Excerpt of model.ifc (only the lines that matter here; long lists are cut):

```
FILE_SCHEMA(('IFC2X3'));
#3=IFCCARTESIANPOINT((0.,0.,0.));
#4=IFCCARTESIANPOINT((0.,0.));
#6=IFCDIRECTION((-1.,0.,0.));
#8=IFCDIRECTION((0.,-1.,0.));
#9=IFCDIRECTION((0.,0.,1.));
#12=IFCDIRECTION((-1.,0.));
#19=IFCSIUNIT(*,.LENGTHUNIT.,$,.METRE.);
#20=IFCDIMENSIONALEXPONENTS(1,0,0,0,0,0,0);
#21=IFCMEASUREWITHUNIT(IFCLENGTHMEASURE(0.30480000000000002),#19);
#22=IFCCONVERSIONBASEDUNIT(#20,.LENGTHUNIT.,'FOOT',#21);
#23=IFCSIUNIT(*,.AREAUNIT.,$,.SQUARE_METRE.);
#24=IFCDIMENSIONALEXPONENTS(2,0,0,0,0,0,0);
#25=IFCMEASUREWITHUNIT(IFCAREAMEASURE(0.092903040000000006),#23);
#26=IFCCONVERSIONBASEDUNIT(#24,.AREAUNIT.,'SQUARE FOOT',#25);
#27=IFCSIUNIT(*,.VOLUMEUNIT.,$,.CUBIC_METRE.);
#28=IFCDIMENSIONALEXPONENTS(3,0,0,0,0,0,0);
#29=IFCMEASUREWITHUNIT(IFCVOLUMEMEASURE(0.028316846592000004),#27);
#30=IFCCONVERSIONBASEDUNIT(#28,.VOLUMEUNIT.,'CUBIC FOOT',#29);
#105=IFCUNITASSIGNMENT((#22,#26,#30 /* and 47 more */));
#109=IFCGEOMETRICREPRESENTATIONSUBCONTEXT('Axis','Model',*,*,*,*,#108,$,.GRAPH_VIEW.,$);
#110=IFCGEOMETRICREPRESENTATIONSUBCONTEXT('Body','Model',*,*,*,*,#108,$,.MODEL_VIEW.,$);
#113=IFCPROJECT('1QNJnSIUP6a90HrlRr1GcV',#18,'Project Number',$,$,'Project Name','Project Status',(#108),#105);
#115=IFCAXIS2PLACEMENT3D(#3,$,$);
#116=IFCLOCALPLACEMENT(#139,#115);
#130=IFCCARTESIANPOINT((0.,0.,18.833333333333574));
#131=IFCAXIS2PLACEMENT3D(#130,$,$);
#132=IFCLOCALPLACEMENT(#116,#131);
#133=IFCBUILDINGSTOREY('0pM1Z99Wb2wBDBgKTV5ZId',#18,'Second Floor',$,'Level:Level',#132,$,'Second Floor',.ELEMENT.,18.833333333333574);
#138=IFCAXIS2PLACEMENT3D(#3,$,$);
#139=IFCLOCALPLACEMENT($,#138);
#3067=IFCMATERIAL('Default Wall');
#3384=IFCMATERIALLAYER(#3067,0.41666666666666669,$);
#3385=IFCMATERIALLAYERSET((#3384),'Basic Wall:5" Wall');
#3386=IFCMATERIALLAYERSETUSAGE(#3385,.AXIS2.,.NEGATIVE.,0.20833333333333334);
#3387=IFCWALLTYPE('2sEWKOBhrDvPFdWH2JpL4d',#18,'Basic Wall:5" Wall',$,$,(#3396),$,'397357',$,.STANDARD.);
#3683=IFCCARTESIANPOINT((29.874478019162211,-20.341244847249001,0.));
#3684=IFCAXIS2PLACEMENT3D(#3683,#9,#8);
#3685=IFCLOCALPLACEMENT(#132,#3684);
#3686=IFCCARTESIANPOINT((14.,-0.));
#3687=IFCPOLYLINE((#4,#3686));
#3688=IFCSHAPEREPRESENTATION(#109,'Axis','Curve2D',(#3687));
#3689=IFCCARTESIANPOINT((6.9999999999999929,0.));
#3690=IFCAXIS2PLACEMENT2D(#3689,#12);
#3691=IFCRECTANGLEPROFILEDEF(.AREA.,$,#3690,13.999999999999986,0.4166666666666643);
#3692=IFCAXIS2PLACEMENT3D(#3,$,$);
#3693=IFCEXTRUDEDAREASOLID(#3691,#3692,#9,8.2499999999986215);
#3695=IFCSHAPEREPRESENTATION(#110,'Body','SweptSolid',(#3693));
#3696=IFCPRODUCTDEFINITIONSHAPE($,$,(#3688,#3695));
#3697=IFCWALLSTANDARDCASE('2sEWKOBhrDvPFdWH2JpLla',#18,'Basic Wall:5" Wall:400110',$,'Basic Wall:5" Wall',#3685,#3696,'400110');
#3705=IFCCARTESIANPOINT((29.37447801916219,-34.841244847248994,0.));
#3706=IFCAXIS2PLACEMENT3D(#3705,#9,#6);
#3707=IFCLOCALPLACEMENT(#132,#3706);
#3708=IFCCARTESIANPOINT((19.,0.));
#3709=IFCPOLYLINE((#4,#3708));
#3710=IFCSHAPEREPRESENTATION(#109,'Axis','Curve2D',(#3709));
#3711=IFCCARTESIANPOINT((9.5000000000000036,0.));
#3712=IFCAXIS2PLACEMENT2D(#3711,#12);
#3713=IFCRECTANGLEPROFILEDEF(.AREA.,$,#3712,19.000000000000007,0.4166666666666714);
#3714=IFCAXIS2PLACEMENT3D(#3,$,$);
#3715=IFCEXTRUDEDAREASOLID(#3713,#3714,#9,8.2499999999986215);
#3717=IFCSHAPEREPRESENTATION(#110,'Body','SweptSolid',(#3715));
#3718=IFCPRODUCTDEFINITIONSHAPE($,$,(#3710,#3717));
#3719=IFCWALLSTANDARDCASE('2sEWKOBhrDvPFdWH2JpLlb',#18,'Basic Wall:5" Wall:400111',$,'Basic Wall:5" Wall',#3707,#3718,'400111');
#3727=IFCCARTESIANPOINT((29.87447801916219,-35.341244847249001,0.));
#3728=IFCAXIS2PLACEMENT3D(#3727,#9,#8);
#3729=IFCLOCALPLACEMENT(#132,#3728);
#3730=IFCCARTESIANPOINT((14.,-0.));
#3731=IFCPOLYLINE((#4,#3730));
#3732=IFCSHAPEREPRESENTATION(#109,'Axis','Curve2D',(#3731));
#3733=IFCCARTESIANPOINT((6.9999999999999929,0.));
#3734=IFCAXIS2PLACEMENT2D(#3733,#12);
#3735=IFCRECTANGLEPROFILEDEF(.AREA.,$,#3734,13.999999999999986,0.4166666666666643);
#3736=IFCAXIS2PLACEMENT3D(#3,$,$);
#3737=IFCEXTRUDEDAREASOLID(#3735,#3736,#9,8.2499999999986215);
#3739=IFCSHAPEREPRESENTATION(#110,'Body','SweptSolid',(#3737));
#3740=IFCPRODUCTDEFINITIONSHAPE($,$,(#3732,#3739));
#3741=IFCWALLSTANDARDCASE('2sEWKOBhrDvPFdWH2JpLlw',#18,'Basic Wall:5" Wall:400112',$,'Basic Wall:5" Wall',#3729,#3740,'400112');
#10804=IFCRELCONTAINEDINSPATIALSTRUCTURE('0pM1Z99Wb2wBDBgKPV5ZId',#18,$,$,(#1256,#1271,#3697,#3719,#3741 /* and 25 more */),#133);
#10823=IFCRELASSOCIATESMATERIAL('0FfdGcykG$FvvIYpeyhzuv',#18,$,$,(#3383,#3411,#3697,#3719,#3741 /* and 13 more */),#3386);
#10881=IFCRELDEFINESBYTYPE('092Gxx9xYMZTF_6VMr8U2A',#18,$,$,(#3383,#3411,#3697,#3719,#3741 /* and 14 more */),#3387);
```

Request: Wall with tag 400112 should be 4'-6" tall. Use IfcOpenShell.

```python
import ifcopenshell
import ifcopenshell.geom
import ifcopenshell.util.representation
import ifcopenshell.util.shape
import ifcopenshell.util.unit

model = ifcopenshell.open("model.ifc")
unit_scale = ifcopenshell.util.unit.calculate_unit_scale(model)
settings = ifcopenshell.geom.settings()


def volume(element):
    """Net volume in cubic metres, openings subtracted."""
    shape = ifcopenshell.geom.create_shape(settings, element)
    return ifcopenshell.util.shape.get_volume(shape.geometry)


wall = model.by_id(3741)
before = volume(wall)

body = ifcopenshell.util.representation.get_representation(wall, "Model", "Body")
solid = body.Items[0]
old_height = solid.Depth
solid.Depth = 54 * 0.0254 / unit_scale
after = volume(wall)

print(f"height {old_height:g} -> {solid.Depth:g}, volume {before:.3f} -> {after:.3f} m3")

model.write("model_edited.ifc")
```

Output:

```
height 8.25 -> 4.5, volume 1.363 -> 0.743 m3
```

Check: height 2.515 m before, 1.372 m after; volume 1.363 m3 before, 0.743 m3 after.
